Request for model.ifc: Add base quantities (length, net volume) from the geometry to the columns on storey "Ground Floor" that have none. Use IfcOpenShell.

First a look at what the model holds.

```python
import ifcopenshell
import ifcopenshell.util.element
import ifcopenshell.util.unit

model = ifcopenshell.open("model.ifc")
print(model.schema)
for unit_type in ("LENGTHUNIT", "AREAUNIT", "VOLUMEUNIT"):
    print(unit_type, ifcopenshell.util.unit.calculate_unit_scale(model, unit_type))
storey = next(s for s in model.by_type("IfcBuildingStorey") if s.Name == "Ground Floor")
columns = [e for e in ifcopenshell.util.element.get_decomposition(storey) if e.is_a("IfcColumn")]
for e in sorted(columns, key=lambda e: e.id()):
    print(e.id(), e.is_a(), e.Name, list(ifcopenshell.util.element.get_psets(e, qtos_only=True)), sep=" | ")
```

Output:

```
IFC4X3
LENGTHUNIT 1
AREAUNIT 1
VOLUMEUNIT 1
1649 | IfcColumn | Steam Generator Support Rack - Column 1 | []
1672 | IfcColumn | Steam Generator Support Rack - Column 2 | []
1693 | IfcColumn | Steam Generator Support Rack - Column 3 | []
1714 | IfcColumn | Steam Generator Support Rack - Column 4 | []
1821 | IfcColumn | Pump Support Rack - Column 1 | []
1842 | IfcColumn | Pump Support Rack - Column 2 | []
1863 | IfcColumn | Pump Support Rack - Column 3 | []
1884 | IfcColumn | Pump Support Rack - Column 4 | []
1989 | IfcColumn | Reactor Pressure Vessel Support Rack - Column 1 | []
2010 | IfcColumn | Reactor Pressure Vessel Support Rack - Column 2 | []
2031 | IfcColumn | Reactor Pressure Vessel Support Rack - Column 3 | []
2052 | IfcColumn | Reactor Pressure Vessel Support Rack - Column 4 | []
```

```python
import ifcopenshell
import ifcopenshell.api.pset
import ifcopenshell.geom
import ifcopenshell.util.element
import ifcopenshell.util.shape
import ifcopenshell.util.unit

model = ifcopenshell.open("model.ifc")
unit_scale = ifcopenshell.util.unit.calculate_unit_scale(model)
volume_scale = ifcopenshell.util.unit.calculate_unit_scale(model, "VOLUMEUNIT")
settings = ifcopenshell.geom.settings()

storey = next(s for s in model.by_type("IfcBuildingStorey") if s.Name == "Ground Floor")
columns = [e for e in ifcopenshell.util.element.get_decomposition(storey) if e.is_a("IfcColumn")]

for e in sorted(columns, key=lambda e: e.id()):
    if ifcopenshell.util.element.get_psets(e, qtos_only=True, should_inherit=False):
        continue
    # Geometry comes back in metres, in the element's own axes.
    shape = ifcopenshell.geom.create_shape(settings, e)
    values = {
        "Length": ifcopenshell.util.shape.get_z(shape.geometry) / unit_scale,
        "NetVolume": ifcopenshell.util.shape.get_volume(shape.geometry) / volume_scale,
    }
    qto = ifcopenshell.api.pset.add_qto(model, product=e, name="Qto_ColumnBaseQuantities")
    ifcopenshell.api.pset.edit_qto(model, qto=qto, properties=values)
    print(e.id(), {k: round(v, 3) for k, v in values.items()})

model.write("model_rev.ifc")
```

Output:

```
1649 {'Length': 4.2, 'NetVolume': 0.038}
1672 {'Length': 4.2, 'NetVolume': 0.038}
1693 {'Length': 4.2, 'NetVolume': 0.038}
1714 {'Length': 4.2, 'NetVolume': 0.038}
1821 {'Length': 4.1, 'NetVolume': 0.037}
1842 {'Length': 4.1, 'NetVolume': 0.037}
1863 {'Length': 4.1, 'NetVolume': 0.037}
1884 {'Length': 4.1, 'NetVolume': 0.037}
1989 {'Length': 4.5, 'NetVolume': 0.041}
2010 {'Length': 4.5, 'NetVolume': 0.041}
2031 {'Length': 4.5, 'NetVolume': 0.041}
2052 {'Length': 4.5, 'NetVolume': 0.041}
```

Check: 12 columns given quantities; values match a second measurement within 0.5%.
